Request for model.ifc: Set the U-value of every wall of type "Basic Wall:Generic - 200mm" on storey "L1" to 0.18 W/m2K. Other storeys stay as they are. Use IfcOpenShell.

First a look at what the model holds.

```python
import ifcopenshell
import ifcopenshell.util.element

model = ifcopenshell.open("model.ifc")
print(model.schema)
storey = next(s for s in model.by_type("IfcBuildingStorey") if s.Name == "L1")
walls = [e for e in ifcopenshell.util.element.get_decomposition(storey) if e.is_a("IfcWall")]
seen = {}
for e in walls:
    element_type = ifcopenshell.util.element.get_type(e)
    key = (element_type.Name if element_type != e and element_type else None, ifcopenshell.util.element.get_pset(e, "Pset_WallCommon", "ThermalTransmittance"))
    seen[key] = seen.get(key, 0) + 1
for (name, value), count in sorted(seen.items(), key=str):
    print(count, "x", name, "|", value)
```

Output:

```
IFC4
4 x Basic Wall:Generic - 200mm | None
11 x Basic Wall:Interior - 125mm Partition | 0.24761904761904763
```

```python
import ifcopenshell
import ifcopenshell.api.pset
import ifcopenshell.util.element

model = ifcopenshell.open("model.ifc")

storey = next(s for s in model.by_type("IfcBuildingStorey") if s.Name == "L1")
walls = [e for e in ifcopenshell.util.element.get_decomposition(storey) if e.is_a("IfcWall")]

count = 0
for e in walls:
    element_type = ifcopenshell.util.element.get_type(e)
    if element_type in (None, e) or element_type.Name != "Basic Wall:Generic - 200mm":
        continue
    # add_pset returns the element's existing set when there is one.
    pset = ifcopenshell.api.pset.add_pset(model, product=e, name="Pset_WallCommon")
    ifcopenshell.api.pset.edit_pset(model, pset=pset, properties={"ThermalTransmittance": 0.18})
    count += 1

print(count, "walls updated")

model.write("model-out.ifc")
```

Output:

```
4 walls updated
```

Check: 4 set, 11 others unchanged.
